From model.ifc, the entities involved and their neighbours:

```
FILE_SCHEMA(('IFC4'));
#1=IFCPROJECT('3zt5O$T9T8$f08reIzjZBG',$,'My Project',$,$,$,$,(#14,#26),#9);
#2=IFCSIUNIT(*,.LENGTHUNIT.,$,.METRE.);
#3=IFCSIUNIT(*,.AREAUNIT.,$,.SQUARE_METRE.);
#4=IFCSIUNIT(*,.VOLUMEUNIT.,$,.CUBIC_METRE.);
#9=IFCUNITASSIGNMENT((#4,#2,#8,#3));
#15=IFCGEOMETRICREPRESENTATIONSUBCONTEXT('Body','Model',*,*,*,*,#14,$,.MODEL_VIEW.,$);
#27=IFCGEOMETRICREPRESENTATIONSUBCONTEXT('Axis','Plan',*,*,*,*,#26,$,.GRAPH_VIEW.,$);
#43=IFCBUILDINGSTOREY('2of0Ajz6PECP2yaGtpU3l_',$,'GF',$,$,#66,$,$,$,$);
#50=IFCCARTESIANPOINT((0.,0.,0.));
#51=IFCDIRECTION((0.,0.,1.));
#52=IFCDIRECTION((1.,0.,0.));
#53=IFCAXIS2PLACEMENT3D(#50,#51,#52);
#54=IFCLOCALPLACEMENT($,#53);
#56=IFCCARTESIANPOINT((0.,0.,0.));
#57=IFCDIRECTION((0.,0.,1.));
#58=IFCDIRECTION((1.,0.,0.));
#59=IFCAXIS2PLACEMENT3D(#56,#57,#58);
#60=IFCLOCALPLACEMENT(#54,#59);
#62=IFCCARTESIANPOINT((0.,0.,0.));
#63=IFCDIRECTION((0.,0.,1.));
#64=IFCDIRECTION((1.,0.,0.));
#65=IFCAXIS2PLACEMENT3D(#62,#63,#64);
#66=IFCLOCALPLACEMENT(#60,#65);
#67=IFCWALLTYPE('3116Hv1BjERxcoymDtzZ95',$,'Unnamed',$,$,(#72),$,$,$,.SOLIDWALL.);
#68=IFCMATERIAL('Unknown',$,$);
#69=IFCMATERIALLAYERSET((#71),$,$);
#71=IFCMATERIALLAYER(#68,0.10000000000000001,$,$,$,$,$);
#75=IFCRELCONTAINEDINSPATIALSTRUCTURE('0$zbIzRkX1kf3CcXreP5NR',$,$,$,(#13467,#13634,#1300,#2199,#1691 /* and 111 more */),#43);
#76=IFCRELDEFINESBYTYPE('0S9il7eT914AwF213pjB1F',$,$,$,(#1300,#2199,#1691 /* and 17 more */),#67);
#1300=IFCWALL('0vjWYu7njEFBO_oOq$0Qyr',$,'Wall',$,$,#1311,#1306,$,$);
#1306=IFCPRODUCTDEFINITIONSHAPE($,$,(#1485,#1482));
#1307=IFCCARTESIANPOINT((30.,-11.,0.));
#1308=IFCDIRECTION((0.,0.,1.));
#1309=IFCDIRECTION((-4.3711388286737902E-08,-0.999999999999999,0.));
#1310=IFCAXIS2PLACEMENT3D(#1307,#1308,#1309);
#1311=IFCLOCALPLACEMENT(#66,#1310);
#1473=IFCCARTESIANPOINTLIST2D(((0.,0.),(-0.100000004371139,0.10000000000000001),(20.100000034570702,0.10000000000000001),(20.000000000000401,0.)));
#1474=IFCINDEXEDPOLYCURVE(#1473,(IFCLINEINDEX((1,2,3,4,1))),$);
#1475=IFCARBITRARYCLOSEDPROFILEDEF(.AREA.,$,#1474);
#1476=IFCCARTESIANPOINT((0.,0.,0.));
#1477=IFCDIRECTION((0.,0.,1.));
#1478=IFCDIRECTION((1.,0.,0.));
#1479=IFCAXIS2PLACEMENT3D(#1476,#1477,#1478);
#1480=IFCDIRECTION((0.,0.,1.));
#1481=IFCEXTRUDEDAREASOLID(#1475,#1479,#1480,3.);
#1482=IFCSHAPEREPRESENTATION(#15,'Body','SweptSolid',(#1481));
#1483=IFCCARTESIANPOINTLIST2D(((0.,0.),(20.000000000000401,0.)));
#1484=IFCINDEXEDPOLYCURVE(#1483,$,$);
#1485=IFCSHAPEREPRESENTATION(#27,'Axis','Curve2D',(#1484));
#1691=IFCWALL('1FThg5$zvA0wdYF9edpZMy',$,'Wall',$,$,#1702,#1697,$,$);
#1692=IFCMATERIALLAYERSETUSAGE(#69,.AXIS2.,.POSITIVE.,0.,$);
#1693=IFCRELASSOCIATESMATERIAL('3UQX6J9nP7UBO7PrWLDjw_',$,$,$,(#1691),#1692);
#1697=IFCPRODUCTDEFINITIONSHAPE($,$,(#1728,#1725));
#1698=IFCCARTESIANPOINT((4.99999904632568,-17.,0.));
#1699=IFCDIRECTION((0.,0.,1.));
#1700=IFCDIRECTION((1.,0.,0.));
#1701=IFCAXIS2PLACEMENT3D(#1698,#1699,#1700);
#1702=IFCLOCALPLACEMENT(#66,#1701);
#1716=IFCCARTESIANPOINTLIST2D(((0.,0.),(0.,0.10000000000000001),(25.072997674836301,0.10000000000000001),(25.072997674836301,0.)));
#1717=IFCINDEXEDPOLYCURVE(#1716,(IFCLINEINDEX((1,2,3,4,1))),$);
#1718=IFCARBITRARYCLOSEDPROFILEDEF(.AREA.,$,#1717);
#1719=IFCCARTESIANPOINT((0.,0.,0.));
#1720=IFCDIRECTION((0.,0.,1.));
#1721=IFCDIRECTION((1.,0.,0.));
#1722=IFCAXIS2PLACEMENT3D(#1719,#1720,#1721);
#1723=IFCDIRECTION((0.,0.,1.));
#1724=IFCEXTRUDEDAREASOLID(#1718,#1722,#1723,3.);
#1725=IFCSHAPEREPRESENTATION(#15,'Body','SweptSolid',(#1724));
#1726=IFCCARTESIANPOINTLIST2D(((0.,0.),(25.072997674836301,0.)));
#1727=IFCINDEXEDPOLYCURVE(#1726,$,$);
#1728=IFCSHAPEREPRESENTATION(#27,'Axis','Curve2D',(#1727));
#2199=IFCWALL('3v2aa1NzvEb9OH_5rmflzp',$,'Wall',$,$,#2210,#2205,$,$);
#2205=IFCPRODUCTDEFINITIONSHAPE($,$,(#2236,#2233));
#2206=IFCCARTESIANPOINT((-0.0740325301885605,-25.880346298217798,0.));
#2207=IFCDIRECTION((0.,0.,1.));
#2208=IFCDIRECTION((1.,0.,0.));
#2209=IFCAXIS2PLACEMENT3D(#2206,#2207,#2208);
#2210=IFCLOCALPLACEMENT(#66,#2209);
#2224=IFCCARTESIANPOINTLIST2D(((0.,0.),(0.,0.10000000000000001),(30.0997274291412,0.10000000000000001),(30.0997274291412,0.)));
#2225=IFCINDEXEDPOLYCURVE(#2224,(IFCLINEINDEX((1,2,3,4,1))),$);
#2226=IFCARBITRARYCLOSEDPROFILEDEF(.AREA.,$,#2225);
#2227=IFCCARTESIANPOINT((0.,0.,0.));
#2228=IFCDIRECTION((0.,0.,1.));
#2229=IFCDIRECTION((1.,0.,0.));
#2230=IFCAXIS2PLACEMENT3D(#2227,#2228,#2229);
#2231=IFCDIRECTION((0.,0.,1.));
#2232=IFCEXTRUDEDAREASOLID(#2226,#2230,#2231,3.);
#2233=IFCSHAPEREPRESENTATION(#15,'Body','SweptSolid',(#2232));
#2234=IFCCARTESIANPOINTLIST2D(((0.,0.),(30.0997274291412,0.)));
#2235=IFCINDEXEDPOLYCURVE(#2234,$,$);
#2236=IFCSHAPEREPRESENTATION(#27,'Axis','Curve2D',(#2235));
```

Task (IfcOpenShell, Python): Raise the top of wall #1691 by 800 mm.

```python
import ifcopenshell
import ifcopenshell.geom
import ifcopenshell.util.representation
import ifcopenshell.util.shape
import ifcopenshell.util.unit

model = ifcopenshell.open("model.ifc")
unit_scale = ifcopenshell.util.unit.calculate_unit_scale(model)
settings = ifcopenshell.geom.settings()


def volume(element):
    """Net volume in cubic metres, openings subtracted."""
    shape = ifcopenshell.geom.create_shape(settings, element)
    return ifcopenshell.util.shape.get_volume(shape.geometry)


wall = model.by_guid("1FThg5$zvA0wdYF9edpZMy")
before = volume(wall)

body = ifcopenshell.util.representation.get_representation(wall, "Model", "Body")
solid = body.Items[0]
old_height = solid.Depth
solid.Depth += 0.8 / unit_scale
after = volume(wall)

print(f"height {old_height:g} -> {solid.Depth:g}, volume {before:.3f} -> {after:.3f} m3")

model.write("model-out.ifc")
```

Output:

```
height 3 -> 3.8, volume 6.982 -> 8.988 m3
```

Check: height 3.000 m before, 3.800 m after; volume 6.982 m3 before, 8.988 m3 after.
